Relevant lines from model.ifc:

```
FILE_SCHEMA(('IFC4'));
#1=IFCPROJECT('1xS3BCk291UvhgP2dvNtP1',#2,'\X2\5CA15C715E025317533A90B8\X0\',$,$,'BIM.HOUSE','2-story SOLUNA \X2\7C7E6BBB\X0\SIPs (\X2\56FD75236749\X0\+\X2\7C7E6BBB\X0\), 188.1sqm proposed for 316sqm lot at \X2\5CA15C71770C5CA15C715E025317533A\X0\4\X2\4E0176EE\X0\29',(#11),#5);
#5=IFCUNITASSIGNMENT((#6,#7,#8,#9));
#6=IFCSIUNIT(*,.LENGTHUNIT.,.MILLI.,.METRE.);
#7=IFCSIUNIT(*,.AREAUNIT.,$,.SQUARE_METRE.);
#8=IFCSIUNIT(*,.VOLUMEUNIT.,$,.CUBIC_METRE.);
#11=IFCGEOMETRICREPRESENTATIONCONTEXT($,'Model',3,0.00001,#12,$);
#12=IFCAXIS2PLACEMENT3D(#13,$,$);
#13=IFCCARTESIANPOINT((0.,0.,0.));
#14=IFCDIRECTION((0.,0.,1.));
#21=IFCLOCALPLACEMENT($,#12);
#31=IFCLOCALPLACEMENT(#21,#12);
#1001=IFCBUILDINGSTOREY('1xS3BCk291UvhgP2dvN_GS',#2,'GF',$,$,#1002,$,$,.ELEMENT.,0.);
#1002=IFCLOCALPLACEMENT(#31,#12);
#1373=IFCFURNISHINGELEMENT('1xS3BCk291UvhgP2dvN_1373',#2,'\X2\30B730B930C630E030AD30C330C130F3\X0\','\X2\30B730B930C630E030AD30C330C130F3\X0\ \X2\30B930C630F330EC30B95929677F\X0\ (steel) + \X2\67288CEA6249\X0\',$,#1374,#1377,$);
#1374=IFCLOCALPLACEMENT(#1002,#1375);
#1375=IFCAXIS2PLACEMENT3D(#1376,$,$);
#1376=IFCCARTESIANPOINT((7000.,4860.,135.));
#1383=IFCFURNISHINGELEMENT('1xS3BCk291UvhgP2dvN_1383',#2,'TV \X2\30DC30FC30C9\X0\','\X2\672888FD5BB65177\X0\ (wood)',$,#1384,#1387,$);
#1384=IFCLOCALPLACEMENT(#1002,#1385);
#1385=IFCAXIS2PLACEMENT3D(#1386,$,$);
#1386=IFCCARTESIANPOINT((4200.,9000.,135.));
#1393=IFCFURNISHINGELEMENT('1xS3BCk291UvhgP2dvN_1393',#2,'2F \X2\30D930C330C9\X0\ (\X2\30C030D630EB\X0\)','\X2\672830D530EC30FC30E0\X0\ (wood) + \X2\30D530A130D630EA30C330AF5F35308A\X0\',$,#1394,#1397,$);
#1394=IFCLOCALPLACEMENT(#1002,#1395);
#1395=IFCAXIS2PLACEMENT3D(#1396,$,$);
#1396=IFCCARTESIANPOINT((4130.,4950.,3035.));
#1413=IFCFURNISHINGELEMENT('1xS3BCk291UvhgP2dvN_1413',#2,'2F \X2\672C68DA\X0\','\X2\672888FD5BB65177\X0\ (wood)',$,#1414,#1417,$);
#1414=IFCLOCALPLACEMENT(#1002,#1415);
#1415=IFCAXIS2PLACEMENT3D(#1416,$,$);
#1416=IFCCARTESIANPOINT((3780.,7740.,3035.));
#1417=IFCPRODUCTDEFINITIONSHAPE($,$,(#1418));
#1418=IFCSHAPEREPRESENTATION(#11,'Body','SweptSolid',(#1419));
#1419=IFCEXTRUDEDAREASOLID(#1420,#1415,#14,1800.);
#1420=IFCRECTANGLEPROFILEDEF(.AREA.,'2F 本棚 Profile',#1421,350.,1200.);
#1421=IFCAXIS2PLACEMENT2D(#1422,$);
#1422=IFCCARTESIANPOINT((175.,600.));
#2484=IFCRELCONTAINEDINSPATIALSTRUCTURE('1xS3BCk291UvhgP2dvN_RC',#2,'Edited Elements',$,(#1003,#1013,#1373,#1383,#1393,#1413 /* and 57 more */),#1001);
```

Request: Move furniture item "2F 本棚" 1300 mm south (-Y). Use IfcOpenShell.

```python
import ifcopenshell
import ifcopenshell.api.geometry
import ifcopenshell.util.placement
import ifcopenshell.util.unit

model = ifcopenshell.open("model.ifc")
unit_scale = ifcopenshell.util.unit.calculate_unit_scale(model)

item = model.by_guid("1xS3BCk291UvhgP2dvN_1413")
matrix = ifcopenshell.util.placement.get_local_placement(item.ObjectPlacement)
matrix[1, 3] -= 1.3 / unit_scale
ifcopenshell.api.geometry.edit_object_placement(model, product=item, matrix=matrix, is_si=False)

print(ifcopenshell.util.placement.get_local_placement(item.ObjectPlacement).round(3) + 0.0)

model.write("model_v2.ifc")
```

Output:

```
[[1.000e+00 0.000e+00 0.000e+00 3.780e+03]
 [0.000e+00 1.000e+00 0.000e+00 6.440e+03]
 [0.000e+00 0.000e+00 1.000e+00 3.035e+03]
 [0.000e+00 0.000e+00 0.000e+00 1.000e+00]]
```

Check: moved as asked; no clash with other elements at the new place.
